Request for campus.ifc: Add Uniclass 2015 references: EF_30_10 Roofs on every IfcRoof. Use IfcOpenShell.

First a look at what the model holds.

```python
import ifcopenshell

model = ifcopenshell.open("campus.ifc")
print(model.schema)
print("classifications:", [c.Name for c in model.by_type("IfcClassification")])
for ifc_class in ("IfcDoor", "IfcRoof", "IfcStair", "IfcWall", "IfcWindow"):
    print(ifc_class, len(model.by_type(ifc_class)))
```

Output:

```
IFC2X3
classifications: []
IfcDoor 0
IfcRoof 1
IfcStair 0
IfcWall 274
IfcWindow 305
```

```python
import ifcopenshell
import ifcopenshell.api.classification

model = ifcopenshell.open("campus.ifc")

# IFC2X3 requires Source and Edition and has no link from the project to the system.
system = model.create_entity("IfcClassification", Source="NBS", Edition="2015", Name="Uniclass 2015")

codes = {
    "IfcRoof": ("EF_30_10", "Roofs"),
}
for ifc_class, (code, name) in codes.items():
    products = model.by_type(ifc_class)
    ifcopenshell.api.classification.add_reference(
        model, products=products, classification=system, identification=code, name=name
    )
    print(code, len(products))

model.write("campus-out.ifc")
```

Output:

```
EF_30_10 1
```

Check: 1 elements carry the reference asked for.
